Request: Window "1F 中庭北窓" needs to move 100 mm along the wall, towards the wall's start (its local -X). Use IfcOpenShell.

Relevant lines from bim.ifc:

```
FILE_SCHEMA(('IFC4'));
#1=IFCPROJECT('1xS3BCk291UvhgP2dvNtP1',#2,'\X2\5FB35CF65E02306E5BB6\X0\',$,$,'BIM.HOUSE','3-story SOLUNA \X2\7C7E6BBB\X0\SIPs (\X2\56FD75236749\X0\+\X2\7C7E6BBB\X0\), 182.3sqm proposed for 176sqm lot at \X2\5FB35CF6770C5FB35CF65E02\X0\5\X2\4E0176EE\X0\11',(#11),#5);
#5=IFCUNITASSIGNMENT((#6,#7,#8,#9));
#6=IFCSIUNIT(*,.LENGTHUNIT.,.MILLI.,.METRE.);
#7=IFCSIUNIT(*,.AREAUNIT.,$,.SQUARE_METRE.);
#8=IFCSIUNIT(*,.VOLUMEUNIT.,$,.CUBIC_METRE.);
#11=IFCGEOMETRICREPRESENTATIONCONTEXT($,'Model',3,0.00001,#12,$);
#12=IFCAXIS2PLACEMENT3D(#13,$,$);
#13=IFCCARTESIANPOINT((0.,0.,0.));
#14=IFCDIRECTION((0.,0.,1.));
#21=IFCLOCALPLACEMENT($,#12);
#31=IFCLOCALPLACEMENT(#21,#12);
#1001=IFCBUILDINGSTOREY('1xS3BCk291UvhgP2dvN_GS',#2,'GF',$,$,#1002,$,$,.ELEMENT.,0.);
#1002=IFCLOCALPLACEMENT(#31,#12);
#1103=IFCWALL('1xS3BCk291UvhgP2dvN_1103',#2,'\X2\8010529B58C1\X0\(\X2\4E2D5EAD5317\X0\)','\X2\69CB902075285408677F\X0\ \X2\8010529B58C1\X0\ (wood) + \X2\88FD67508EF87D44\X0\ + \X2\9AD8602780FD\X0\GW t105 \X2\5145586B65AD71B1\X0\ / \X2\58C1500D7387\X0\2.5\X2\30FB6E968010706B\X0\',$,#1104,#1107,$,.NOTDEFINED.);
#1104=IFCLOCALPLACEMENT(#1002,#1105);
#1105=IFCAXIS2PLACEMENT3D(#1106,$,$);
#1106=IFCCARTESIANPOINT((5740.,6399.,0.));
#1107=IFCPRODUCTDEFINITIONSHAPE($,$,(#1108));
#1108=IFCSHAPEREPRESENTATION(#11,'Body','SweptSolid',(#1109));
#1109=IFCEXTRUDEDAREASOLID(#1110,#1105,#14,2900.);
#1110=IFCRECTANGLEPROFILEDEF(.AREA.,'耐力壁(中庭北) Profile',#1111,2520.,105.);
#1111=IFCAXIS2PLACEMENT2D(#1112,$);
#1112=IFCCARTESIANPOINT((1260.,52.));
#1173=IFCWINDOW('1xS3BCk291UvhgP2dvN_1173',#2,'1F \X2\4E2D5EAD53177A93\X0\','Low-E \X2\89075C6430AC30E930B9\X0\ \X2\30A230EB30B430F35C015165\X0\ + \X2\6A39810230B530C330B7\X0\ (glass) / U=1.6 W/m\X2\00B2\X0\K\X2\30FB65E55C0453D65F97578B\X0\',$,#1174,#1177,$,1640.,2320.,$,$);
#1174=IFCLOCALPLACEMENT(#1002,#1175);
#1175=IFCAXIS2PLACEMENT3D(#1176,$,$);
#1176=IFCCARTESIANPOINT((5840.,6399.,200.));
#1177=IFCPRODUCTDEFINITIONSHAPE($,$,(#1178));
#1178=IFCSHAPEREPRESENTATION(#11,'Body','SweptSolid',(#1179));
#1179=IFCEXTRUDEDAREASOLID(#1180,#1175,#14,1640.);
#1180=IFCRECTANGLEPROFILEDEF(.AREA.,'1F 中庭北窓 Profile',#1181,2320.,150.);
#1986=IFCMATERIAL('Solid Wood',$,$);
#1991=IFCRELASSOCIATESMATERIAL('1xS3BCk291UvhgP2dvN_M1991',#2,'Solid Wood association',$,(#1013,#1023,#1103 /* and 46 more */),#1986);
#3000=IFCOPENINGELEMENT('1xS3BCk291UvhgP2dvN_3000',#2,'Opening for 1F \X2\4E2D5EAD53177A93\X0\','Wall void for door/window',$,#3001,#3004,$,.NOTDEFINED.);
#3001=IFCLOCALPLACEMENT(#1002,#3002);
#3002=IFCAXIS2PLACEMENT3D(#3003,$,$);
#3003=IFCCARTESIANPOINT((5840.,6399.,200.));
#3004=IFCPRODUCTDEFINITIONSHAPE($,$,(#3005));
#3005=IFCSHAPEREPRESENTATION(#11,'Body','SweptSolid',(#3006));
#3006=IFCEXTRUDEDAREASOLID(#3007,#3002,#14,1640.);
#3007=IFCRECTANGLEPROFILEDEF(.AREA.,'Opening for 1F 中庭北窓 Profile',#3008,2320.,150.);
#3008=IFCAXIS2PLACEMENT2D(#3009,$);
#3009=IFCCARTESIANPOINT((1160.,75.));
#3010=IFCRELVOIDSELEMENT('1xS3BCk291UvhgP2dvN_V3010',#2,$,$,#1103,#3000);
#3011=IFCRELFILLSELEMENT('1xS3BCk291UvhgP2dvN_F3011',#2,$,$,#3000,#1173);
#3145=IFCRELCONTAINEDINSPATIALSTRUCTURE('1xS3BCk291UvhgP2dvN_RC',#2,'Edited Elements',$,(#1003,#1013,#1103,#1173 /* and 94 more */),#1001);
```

```python
import ifcopenshell
import ifcopenshell.api.geometry
import ifcopenshell.util.placement
import ifcopenshell.util.unit

model = ifcopenshell.open("bim.ifc")
unit_scale = ifcopenshell.util.unit.calculate_unit_scale(model)

window = model.by_guid("1xS3BCk291UvhgP2dvN_1173")
opening = window.FillsVoids[0].RelatingOpeningElement
wall = opening.VoidsElements[0].RelatingBuildingElement

wall_matrix = ifcopenshell.util.placement.get_local_placement(wall.ObjectPlacement)
shift = wall_matrix[:3, 0] * -0.1 / unit_scale
before = ifcopenshell.util.placement.get_local_placement(window.ObjectPlacement)[:3, 3].copy()

# The window is not placed relative to its opening, so move both.
for product in (opening, window):
    matrix = ifcopenshell.util.placement.get_local_placement(product.ObjectPlacement)
    matrix[:3, 3] += shift
    ifcopenshell.api.geometry.edit_object_placement(model, product=product, matrix=matrix, is_si=False)

after = ifcopenshell.util.placement.get_local_placement(window.ObjectPlacement)[:3, 3]
print("window moved by", (after - before).round(3) + 0.0)

model.write("bim_updated.ifc")
```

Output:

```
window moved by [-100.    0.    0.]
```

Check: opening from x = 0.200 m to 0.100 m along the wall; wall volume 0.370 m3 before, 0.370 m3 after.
